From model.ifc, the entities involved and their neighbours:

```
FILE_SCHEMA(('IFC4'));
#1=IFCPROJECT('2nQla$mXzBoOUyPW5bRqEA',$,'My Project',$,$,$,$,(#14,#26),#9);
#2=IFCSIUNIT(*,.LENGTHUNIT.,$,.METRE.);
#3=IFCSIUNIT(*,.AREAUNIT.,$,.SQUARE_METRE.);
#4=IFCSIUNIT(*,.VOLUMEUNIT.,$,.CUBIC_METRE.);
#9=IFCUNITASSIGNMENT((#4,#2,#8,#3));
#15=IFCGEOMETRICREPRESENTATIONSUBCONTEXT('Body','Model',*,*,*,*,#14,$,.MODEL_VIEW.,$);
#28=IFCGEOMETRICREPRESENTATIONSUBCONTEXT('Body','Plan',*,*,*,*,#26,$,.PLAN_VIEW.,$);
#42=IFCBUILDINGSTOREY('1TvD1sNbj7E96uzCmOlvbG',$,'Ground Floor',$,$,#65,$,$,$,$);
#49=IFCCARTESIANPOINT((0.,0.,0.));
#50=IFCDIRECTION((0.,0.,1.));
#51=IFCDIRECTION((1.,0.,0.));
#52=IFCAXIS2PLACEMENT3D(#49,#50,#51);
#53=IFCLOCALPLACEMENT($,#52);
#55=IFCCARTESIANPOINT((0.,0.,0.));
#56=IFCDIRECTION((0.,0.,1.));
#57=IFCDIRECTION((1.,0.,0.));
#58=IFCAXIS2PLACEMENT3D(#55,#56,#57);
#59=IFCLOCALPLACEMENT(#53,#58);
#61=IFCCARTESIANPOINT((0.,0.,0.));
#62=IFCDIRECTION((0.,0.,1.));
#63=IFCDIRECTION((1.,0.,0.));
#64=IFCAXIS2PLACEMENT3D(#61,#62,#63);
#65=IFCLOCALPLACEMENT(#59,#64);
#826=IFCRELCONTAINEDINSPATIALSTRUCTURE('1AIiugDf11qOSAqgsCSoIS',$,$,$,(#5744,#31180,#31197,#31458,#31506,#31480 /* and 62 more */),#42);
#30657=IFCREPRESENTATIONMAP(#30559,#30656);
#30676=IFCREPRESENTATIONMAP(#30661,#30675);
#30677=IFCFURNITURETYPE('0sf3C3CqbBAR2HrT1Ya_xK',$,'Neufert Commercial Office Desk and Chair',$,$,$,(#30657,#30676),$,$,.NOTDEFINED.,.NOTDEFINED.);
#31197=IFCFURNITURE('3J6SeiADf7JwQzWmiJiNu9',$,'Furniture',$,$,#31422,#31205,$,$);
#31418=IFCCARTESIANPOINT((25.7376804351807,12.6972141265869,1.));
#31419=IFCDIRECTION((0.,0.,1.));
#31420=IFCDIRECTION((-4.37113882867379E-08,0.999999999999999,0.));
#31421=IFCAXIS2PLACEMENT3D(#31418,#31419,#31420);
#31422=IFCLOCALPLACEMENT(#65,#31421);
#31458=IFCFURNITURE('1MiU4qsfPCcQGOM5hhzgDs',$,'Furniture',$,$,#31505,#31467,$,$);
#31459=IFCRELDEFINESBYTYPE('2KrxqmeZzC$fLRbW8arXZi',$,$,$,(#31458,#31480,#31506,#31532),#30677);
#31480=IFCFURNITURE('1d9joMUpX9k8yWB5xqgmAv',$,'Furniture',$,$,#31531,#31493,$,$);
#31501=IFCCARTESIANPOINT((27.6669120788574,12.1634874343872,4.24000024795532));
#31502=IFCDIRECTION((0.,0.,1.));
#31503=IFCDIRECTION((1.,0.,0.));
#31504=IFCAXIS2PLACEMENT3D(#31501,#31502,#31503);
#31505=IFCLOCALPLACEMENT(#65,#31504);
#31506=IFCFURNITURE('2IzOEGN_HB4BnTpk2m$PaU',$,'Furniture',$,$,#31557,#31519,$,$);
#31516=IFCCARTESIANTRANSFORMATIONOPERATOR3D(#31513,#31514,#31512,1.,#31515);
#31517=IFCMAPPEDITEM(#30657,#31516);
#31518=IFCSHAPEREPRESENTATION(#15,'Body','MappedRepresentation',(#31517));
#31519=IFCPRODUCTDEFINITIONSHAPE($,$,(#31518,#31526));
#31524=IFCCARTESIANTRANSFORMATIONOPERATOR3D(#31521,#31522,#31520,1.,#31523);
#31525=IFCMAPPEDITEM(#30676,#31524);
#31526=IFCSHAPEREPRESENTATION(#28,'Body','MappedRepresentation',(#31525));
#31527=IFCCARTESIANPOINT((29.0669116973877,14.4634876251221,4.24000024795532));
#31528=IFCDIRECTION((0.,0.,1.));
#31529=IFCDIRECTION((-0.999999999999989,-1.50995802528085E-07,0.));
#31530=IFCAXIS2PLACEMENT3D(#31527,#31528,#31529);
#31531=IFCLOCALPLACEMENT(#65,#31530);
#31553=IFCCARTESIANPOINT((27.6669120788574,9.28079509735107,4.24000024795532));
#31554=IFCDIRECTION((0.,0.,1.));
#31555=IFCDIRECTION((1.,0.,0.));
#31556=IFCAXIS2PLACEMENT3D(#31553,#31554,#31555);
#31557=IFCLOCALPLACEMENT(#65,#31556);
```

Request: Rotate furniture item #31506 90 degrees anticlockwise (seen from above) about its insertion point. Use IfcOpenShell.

```python
import ifcopenshell
import ifcopenshell.api.geometry
import ifcopenshell.util.placement

model = ifcopenshell.open("model.ifc")

item = model.by_guid("2IzOEGN_HB4BnTpk2m$PaU")
matrix = ifcopenshell.util.placement.get_local_placement(item.ObjectPlacement)
matrix = matrix @ ifcopenshell.util.placement.rotation(90, "Z")
ifcopenshell.api.geometry.edit_object_placement(model, product=item, matrix=matrix, is_si=False)

print(ifcopenshell.util.placement.get_local_placement(item.ObjectPlacement).round(3) + 0.0)

model.write("model_updated.ifc")
```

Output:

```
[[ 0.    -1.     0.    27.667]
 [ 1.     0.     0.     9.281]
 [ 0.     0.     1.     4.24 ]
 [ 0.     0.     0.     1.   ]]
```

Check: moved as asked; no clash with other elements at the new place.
